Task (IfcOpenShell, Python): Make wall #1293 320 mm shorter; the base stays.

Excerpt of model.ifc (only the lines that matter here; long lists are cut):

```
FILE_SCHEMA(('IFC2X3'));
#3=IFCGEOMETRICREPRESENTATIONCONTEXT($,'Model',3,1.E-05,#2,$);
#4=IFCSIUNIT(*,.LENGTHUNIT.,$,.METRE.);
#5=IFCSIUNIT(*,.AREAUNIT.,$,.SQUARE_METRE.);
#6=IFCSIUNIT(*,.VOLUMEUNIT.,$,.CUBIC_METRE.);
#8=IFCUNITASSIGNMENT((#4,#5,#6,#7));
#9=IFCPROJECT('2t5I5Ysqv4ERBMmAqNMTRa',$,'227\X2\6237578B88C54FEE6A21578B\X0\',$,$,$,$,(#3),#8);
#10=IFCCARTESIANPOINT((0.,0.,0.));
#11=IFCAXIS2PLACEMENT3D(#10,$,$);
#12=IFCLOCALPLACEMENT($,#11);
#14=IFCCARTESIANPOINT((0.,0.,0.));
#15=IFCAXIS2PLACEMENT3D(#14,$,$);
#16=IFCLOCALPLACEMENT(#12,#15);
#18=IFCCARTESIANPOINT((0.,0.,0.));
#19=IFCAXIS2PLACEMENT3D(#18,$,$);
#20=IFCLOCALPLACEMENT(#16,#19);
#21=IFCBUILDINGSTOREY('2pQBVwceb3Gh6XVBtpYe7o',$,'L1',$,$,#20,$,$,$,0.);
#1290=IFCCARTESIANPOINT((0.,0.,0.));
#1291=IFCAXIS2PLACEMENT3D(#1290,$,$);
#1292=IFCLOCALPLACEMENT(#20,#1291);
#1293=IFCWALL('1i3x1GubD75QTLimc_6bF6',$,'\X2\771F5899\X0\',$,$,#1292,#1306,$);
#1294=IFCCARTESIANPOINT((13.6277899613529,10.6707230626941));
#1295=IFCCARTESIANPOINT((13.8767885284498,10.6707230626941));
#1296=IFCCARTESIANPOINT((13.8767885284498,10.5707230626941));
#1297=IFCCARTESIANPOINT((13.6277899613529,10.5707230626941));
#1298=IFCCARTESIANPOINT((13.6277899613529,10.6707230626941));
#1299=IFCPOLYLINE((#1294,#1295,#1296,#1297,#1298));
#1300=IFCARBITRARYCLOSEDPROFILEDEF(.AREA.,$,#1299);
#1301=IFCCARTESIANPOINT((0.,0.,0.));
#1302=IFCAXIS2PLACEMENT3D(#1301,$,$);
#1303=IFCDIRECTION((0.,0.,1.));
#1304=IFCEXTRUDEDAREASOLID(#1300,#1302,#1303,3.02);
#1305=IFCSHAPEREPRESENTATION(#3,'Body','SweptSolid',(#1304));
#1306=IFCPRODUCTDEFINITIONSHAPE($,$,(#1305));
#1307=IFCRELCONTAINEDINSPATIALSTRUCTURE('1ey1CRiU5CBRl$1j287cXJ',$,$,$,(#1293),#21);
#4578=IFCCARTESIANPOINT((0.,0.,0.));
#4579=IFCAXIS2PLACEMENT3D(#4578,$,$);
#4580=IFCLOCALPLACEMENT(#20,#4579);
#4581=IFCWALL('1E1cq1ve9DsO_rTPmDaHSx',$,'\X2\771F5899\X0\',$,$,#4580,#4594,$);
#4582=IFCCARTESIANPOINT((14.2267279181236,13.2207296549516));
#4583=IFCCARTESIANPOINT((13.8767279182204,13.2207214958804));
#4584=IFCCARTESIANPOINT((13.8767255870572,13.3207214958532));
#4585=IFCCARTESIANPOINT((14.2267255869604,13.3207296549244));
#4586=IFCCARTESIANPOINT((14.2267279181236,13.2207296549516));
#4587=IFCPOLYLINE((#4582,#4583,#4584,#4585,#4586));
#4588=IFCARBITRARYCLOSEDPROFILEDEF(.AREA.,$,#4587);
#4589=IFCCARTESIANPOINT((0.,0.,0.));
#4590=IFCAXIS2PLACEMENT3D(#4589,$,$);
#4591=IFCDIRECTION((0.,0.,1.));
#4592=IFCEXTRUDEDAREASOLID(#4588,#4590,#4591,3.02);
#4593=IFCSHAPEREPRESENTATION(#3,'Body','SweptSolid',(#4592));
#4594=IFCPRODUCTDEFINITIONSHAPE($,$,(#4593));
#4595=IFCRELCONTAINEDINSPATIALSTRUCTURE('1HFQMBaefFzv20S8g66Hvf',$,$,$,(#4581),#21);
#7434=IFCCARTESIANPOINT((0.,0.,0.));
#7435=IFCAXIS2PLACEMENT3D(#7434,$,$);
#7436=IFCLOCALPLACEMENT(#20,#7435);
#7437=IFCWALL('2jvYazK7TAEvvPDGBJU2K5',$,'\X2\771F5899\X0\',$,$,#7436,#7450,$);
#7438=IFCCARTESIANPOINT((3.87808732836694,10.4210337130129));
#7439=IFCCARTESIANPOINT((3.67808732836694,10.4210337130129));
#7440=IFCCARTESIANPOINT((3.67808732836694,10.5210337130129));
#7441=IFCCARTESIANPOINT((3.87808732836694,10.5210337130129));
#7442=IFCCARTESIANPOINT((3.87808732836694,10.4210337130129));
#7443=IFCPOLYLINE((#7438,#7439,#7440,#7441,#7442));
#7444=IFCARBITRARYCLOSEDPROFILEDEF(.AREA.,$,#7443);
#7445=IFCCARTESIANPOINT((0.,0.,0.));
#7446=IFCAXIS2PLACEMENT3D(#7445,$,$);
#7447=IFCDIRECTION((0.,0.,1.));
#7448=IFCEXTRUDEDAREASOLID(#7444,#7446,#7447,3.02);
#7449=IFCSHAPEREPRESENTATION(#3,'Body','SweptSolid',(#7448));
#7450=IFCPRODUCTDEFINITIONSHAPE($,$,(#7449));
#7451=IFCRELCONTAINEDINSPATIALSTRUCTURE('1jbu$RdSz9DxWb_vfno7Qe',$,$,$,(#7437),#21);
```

```python
import ifcopenshell
import ifcopenshell.geom
import ifcopenshell.util.shape
import ifcopenshell.util.unit

model = ifcopenshell.open("model.ifc")
unit_scale = ifcopenshell.util.unit.calculate_unit_scale(model)
settings = ifcopenshell.geom.settings()


def volume(element):
    """Net volume in cubic metres, openings subtracted."""
    shape = ifcopenshell.geom.create_shape(settings, element)
    return ifcopenshell.util.shape.get_volume(shape.geometry)


wall = model.by_id(1293)
before = volume(wall)

body = next(r for r in wall.Representation.Representations if r.RepresentationIdentifier == "Body")
solid = body.Items[0]
old_height = solid.Depth
solid.Depth -= 0.32 / unit_scale
after = volume(wall)

print(f"height {old_height:g} -> {solid.Depth:g}, volume {before:.3f} -> {after:.3f} m3")

model.write("model_updated.ifc")
```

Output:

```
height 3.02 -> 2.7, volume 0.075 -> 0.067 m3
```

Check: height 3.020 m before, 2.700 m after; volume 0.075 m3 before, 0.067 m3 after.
